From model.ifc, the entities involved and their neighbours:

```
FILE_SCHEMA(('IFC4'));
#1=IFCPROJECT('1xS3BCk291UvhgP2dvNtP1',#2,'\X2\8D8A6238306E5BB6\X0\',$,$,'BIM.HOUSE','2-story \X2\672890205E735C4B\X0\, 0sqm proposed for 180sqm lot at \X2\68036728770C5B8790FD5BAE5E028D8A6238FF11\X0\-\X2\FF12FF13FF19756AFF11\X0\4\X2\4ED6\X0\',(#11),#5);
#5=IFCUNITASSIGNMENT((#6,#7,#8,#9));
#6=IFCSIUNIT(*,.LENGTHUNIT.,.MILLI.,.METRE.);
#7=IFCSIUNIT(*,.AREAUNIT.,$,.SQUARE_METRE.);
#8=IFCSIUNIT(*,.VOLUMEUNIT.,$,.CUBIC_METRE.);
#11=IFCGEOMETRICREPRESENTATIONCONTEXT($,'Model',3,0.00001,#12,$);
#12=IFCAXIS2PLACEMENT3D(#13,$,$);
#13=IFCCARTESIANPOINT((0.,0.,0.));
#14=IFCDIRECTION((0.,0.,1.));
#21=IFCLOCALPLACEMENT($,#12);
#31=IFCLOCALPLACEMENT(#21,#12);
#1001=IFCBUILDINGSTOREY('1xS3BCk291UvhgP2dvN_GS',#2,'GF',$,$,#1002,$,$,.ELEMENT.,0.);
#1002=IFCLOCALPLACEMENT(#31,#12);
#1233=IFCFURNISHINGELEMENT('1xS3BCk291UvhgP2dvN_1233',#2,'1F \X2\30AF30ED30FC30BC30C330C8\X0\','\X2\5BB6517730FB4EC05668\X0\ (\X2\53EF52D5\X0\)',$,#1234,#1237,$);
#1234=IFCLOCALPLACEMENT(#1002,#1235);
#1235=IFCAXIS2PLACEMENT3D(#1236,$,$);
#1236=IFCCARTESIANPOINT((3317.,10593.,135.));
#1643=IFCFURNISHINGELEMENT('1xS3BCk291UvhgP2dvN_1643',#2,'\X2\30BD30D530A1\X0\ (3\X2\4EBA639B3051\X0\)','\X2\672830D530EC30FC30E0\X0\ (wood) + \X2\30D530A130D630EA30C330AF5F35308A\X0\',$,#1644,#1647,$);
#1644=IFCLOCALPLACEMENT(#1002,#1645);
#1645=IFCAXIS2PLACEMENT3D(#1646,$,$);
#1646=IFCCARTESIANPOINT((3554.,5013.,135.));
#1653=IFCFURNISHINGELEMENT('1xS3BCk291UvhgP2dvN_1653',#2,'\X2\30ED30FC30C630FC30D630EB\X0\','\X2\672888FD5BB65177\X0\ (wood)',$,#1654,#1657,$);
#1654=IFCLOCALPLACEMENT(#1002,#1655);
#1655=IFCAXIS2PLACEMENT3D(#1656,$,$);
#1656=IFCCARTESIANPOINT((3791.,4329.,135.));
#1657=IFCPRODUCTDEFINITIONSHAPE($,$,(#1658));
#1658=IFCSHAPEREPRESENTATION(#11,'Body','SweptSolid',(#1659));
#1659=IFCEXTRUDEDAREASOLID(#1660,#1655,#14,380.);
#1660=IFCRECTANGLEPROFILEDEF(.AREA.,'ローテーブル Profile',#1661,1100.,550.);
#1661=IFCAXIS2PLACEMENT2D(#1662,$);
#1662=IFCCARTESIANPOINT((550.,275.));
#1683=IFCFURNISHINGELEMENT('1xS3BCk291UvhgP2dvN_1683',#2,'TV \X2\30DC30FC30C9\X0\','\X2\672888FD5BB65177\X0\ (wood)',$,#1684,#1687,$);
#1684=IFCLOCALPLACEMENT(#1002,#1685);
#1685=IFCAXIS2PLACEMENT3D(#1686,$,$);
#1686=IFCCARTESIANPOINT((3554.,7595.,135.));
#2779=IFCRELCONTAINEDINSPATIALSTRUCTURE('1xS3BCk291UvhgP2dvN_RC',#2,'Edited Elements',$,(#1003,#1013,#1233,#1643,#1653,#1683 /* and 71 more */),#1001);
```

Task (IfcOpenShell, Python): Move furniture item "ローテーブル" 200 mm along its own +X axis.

```python
import ifcopenshell
import ifcopenshell.api.geometry
import ifcopenshell.util.placement

model = ifcopenshell.open("model.ifc")

item = model.by_guid("1xS3BCk291UvhgP2dvN_1653")
matrix = ifcopenshell.util.placement.get_local_placement(item.ObjectPlacement)
matrix[:3, 3] += matrix[:3, 0] * 200.0
ifcopenshell.api.geometry.edit_object_placement(model, product=item, matrix=matrix, is_si=False)

print(ifcopenshell.util.placement.get_local_placement(item.ObjectPlacement).round(3) + 0.0)

model.write("model-out.ifc")
```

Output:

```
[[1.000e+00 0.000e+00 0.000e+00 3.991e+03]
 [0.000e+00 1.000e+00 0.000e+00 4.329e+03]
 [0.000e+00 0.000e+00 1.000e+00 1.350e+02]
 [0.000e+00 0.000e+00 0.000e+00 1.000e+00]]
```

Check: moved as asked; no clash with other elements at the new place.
